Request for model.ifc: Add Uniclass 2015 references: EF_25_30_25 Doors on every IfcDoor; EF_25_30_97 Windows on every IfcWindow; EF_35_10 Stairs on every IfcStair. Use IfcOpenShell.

First a look at what the model holds.

```python
import ifcopenshell

model = ifcopenshell.open("model.ifc")
print(model.schema)
print("classifications:", [c.Name for c in model.by_type("IfcClassification")])
for ifc_class in ("IfcDoor", "IfcRoof", "IfcStair", "IfcWall", "IfcWindow"):
    print(ifc_class, len(model.by_type(ifc_class)))
```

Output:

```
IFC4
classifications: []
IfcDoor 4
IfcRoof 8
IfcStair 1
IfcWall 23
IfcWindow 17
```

```python
import ifcopenshell
import ifcopenshell.api.classification

model = ifcopenshell.open("model.ifc")

system = ifcopenshell.api.classification.add_classification(model, classification="Uniclass 2015")

codes = {
    "IfcDoor": ("EF_25_30_25", "Doors"),
    "IfcWindow": ("EF_25_30_97", "Windows"),
    "IfcStair": ("EF_35_10", "Stairs"),
}
for ifc_class, (code, name) in codes.items():
    products = model.by_type(ifc_class)
    ifcopenshell.api.classification.add_reference(
        model, products=products, classification=system, identification=code, name=name
    )
    print(code, len(products))

model.write("model_v2.ifc")
```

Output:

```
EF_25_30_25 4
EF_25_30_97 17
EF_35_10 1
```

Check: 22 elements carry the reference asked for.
